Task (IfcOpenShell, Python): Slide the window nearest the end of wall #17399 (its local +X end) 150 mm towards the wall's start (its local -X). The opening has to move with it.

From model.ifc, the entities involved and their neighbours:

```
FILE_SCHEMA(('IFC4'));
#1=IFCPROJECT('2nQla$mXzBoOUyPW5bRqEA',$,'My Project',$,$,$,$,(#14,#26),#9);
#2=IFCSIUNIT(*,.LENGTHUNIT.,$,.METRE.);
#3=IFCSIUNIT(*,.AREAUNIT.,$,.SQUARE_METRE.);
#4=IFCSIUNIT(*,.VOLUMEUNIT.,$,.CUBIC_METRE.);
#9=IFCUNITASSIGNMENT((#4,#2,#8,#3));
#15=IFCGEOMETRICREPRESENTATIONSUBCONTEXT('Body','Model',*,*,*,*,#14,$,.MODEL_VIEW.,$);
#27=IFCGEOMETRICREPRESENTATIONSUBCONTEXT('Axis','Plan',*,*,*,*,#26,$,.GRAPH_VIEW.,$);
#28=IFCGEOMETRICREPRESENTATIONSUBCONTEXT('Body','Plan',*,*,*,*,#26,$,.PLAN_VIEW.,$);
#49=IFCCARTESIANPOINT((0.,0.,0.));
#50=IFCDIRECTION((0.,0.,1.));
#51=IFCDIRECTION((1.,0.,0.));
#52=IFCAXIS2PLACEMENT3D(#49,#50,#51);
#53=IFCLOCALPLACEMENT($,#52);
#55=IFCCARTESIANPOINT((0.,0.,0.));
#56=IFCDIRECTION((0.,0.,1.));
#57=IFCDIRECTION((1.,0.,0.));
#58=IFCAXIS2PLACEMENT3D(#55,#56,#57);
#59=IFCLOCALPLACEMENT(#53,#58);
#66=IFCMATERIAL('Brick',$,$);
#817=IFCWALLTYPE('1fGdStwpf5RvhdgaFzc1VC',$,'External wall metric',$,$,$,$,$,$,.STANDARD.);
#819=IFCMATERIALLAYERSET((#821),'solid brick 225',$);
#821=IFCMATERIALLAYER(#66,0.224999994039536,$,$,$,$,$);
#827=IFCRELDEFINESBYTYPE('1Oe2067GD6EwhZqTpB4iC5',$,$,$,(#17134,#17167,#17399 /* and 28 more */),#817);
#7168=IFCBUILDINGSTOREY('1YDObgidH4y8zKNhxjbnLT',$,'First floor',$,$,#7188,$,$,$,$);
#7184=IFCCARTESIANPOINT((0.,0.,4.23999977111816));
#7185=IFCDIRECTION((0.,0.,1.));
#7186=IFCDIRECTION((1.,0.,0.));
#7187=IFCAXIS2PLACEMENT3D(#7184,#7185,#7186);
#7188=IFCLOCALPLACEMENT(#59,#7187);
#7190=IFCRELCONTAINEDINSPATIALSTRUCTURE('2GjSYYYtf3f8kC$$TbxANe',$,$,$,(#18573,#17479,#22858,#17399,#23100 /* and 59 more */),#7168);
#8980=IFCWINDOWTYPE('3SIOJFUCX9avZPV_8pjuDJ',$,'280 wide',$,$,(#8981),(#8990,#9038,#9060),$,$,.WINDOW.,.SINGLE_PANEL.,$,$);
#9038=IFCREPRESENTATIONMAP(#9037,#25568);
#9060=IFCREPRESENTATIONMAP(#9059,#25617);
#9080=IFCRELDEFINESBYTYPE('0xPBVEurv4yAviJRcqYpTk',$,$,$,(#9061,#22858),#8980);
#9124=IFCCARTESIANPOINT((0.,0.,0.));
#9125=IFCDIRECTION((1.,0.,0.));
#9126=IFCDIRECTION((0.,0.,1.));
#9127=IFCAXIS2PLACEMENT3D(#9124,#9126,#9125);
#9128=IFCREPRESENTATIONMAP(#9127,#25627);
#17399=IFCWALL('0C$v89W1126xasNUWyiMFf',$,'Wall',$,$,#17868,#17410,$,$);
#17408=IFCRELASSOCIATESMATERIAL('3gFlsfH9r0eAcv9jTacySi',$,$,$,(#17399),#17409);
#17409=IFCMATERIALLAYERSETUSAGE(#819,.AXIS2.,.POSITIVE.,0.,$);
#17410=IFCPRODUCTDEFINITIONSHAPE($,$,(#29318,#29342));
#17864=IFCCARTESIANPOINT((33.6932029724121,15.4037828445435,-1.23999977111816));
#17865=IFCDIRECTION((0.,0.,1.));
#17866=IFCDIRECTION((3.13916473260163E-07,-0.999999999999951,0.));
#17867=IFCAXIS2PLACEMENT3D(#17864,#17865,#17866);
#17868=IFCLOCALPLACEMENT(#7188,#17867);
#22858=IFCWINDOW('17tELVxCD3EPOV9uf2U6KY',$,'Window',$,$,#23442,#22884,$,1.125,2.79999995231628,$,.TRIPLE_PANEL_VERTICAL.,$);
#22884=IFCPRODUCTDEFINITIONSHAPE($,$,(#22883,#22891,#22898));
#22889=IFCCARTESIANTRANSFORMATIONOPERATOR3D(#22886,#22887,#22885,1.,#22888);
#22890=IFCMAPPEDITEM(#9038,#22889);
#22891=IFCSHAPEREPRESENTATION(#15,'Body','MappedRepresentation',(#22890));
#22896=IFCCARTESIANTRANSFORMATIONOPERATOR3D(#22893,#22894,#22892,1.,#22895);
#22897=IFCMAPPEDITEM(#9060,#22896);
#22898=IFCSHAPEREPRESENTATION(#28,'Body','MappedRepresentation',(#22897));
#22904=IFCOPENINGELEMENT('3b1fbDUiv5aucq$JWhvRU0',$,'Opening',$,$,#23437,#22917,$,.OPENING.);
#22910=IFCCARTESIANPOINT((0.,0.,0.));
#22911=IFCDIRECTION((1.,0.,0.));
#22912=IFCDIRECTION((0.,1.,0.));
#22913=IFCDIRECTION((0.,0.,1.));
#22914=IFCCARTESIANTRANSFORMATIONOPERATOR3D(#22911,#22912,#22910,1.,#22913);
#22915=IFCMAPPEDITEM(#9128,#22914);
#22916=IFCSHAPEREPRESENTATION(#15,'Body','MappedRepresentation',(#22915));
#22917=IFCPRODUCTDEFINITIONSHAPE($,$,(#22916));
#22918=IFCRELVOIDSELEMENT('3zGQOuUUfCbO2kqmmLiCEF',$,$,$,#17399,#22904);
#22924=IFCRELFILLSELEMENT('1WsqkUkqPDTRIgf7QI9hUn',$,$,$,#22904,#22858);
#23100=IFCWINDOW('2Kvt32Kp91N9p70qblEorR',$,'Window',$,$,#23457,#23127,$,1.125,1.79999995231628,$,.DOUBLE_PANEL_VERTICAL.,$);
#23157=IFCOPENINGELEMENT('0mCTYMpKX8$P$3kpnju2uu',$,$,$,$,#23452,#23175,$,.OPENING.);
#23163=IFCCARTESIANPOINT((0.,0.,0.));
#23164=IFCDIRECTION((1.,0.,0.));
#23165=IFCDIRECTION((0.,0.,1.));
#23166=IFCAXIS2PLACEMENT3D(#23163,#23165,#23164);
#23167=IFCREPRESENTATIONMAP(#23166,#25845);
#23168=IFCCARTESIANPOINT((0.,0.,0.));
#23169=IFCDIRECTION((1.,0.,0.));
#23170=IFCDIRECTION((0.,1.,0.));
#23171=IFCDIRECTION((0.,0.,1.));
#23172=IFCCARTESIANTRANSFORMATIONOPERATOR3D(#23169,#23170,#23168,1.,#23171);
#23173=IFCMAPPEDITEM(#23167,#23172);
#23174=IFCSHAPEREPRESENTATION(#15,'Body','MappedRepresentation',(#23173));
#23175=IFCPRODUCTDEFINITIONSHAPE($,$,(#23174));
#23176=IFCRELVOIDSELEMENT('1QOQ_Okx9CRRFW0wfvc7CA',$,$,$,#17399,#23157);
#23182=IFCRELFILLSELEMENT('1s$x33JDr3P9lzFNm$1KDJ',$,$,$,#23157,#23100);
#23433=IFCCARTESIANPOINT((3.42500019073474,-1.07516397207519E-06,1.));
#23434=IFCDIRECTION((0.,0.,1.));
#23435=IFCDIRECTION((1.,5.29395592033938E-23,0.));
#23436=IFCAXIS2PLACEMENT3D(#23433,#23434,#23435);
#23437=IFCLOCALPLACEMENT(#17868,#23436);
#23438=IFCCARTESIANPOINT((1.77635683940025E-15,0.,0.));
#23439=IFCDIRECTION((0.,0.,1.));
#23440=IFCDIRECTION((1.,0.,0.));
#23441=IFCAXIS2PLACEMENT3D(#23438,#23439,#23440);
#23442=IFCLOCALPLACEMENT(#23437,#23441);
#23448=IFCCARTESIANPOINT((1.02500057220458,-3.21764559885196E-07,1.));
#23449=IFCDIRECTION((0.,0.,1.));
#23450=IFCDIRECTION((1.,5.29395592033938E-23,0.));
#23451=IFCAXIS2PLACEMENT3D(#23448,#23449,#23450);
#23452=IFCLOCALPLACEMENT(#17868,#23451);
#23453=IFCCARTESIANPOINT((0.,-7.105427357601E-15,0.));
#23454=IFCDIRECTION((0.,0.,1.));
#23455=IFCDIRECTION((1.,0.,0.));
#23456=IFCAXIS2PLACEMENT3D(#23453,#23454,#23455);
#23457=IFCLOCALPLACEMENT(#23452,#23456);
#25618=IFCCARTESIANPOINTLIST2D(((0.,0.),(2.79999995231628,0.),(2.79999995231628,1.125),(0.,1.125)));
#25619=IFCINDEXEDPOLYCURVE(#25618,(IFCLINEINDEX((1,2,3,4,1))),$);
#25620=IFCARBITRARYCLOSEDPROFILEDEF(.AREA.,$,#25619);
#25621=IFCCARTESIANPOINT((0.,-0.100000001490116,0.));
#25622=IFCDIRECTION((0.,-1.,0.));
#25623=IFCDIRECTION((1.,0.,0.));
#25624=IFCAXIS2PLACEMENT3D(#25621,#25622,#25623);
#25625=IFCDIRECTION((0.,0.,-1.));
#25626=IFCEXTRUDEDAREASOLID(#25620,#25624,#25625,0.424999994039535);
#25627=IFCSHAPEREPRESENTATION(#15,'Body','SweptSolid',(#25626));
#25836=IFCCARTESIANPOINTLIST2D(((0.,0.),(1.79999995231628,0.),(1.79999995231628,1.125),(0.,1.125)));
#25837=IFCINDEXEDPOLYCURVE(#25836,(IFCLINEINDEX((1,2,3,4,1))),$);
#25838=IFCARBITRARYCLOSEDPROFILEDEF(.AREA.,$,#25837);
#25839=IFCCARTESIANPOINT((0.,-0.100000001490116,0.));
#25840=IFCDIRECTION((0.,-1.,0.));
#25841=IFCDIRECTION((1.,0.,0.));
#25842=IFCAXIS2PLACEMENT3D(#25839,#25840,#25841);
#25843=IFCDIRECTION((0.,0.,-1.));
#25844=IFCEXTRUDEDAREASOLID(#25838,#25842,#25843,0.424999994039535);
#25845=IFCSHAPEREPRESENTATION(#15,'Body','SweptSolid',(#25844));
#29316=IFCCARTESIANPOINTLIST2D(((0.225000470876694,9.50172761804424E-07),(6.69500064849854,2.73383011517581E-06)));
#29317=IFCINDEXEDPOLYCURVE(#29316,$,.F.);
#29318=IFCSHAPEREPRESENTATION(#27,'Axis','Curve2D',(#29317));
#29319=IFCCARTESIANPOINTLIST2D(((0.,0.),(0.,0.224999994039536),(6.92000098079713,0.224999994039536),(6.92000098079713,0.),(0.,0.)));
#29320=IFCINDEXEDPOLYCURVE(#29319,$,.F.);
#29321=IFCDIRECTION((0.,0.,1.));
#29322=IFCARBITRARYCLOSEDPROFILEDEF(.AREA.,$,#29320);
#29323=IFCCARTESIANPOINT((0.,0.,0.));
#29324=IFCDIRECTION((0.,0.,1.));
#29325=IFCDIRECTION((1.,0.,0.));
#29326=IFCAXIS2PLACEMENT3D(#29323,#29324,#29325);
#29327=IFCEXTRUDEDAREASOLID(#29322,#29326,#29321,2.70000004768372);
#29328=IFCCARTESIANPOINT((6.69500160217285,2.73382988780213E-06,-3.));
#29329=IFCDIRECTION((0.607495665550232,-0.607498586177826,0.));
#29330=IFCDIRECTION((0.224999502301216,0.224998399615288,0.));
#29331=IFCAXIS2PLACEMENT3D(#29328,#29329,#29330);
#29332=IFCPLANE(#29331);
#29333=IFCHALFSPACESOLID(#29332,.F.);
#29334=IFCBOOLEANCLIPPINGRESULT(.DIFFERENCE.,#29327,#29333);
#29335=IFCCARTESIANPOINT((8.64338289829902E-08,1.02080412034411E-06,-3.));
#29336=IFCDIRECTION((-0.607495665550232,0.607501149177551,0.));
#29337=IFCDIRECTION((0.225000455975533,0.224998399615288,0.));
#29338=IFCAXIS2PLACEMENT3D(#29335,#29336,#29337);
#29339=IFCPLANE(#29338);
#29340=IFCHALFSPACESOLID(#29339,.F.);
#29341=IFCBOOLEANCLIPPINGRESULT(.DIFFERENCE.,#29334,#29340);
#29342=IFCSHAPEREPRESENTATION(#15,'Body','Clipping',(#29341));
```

```python
import ifcopenshell
import ifcopenshell.api.geometry
import ifcopenshell.util.placement
import ifcopenshell.util.unit

model = ifcopenshell.open("model.ifc")
unit_scale = ifcopenshell.util.unit.calculate_unit_scale(model)

window = model.by_id(22858)
opening = window.FillsVoids[0].RelatingOpeningElement
wall = opening.VoidsElements[0].RelatingBuildingElement

wall_matrix = ifcopenshell.util.placement.get_local_placement(wall.ObjectPlacement)
shift = wall_matrix[:3, 0] * -0.15 / unit_scale
before = ifcopenshell.util.placement.get_local_placement(window.ObjectPlacement)[:3, 3].copy()

# The window is placed relative to its opening, so it follows when the opening moves.
matrix = ifcopenshell.util.placement.get_local_placement(opening.ObjectPlacement)
matrix[:3, 3] += shift
ifcopenshell.api.geometry.edit_object_placement(
    model, product=opening, matrix=matrix, is_si=False, should_transform_children=True
)

after = ifcopenshell.util.placement.get_local_placement(window.ObjectPlacement)[:3, 3]
print("window moved by", (after - before).round(3) + 0.0)

model.write("model-out.ifc")
```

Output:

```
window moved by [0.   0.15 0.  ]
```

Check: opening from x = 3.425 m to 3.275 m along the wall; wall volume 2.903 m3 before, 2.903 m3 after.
